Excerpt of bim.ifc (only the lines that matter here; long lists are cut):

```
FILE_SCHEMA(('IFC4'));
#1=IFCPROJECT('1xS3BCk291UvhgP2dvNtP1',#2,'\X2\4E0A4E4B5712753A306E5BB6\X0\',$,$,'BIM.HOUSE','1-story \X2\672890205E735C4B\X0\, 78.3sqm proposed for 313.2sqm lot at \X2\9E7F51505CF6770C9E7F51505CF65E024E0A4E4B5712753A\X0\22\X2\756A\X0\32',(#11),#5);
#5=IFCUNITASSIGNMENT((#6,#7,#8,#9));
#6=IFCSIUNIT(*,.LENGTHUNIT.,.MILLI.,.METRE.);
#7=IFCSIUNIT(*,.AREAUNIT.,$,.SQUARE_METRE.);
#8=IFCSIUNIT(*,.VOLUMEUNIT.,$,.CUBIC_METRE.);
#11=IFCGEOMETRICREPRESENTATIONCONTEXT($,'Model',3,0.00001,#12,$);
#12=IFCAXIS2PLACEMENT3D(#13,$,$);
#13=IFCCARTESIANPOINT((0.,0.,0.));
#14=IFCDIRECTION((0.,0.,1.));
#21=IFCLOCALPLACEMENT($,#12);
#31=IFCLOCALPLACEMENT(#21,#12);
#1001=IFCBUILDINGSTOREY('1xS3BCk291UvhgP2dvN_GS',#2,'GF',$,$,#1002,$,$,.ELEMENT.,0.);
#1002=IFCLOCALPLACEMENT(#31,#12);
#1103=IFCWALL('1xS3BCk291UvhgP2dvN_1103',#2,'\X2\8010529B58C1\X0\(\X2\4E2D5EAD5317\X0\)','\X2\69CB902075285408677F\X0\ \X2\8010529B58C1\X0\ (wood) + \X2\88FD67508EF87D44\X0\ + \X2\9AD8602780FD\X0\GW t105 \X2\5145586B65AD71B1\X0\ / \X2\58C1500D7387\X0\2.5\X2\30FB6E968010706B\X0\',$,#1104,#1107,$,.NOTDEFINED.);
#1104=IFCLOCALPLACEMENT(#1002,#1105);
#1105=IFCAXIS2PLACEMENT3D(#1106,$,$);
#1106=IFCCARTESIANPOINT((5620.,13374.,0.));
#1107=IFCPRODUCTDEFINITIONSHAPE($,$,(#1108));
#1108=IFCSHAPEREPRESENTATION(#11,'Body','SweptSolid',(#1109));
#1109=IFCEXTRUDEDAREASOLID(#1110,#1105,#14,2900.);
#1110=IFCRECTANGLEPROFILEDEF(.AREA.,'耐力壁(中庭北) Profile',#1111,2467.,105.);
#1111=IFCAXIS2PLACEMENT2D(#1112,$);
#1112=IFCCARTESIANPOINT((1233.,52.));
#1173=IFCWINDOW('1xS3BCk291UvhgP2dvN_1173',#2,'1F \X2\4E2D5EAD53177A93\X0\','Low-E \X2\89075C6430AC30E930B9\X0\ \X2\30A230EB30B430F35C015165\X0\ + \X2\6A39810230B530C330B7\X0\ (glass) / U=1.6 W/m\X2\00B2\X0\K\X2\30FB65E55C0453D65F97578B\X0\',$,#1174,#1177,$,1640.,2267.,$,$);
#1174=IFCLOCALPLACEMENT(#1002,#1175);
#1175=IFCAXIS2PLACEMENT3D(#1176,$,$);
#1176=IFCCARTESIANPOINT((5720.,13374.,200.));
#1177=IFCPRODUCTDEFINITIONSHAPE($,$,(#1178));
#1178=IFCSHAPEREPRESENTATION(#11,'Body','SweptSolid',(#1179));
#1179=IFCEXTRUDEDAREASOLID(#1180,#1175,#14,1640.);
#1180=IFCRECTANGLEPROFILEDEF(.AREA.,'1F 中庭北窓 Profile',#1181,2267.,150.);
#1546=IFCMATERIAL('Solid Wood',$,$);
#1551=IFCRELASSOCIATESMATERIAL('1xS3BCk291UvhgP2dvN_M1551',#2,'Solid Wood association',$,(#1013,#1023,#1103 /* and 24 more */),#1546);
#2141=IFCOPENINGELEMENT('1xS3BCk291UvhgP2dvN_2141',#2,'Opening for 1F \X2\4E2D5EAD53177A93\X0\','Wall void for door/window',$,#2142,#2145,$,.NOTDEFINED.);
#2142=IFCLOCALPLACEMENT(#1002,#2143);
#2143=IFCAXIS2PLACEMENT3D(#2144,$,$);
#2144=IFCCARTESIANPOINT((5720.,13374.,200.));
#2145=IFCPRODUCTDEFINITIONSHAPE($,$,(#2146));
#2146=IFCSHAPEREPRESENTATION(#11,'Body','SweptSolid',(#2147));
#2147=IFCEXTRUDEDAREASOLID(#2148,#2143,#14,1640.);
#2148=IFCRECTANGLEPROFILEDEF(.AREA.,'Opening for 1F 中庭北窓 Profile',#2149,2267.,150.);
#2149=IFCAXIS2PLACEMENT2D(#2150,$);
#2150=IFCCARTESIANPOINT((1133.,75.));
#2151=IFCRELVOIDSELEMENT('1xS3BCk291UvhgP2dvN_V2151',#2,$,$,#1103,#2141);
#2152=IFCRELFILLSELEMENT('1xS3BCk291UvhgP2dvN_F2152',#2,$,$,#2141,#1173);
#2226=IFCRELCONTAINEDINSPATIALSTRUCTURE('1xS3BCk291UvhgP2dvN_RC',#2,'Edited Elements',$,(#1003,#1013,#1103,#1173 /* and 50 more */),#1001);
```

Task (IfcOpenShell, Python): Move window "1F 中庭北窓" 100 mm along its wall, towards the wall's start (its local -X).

```python
import ifcopenshell
import ifcopenshell.api.geometry
import ifcopenshell.util.placement
import ifcopenshell.util.unit

model = ifcopenshell.open("bim.ifc")
unit_scale = ifcopenshell.util.unit.calculate_unit_scale(model)

window = model.by_guid("1xS3BCk291UvhgP2dvN_1173")
opening = window.FillsVoids[0].RelatingOpeningElement
wall = opening.VoidsElements[0].RelatingBuildingElement

wall_matrix = ifcopenshell.util.placement.get_local_placement(wall.ObjectPlacement)
shift = wall_matrix[:3, 0] * -0.1 / unit_scale
before = ifcopenshell.util.placement.get_local_placement(window.ObjectPlacement)[:3, 3].copy()

# The window is not placed relative to its opening, so move both.
for product in (opening, window):
    matrix = ifcopenshell.util.placement.get_local_placement(product.ObjectPlacement)
    matrix[:3, 3] += shift
    ifcopenshell.api.geometry.edit_object_placement(model, product=product, matrix=matrix, is_si=False)

after = ifcopenshell.util.placement.get_local_placement(window.ObjectPlacement)[:3, 3]
print("window moved by", (after - before).round(3) + 0.0)

model.write("bim-out.ifc")
```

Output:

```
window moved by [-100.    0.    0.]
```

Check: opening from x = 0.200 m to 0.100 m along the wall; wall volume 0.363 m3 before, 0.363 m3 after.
